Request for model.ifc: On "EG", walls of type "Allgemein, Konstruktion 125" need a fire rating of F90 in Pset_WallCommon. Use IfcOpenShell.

First a look at what the model holds.

```python
import ifcopenshell
import ifcopenshell.util.element

model = ifcopenshell.open("model.ifc")
print(model.schema)
storey = next(s for s in model.by_type("IfcBuildingStorey") if s.Name == "EG")
walls = [e for e in ifcopenshell.util.element.get_decomposition(storey) if e.is_a("IfcWall")]
seen = {}
for e in walls:
    element_type = ifcopenshell.util.element.get_type(e)
    key = (element_type.Name if element_type != e and element_type else None, ifcopenshell.util.element.get_pset(e, "Pset_WallCommon", "FireRating"))
    seen[key] = seen.get(key, 0) + 1
for (name, value), count in sorted(seen.items(), key=str):
    print(count, "x", name, "|", value)
```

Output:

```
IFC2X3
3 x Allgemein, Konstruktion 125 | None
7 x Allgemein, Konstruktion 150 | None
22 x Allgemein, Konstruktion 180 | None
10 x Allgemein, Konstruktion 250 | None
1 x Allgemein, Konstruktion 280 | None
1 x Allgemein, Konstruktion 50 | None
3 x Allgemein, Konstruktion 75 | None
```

```python
import ifcopenshell
import ifcopenshell.api.pset
import ifcopenshell.util.element

model = ifcopenshell.open("model.ifc")

storey = next(s for s in model.by_type("IfcBuildingStorey") if s.Name == "EG")
walls = [e for e in ifcopenshell.util.element.get_decomposition(storey) if e.is_a("IfcWall")]

count = 0
for e in walls:
    element_type = ifcopenshell.util.element.get_type(e)
    if element_type in (None, e) or element_type.Name != "Allgemein, Konstruktion 125":
        continue
    # add_pset returns the element's existing set when there is one.
    pset = ifcopenshell.api.pset.add_pset(model, product=e, name="Pset_WallCommon")
    ifcopenshell.api.pset.edit_pset(model, pset=pset, properties={"FireRating": "F90"})
    count += 1

print(count, "walls updated")

model.write("model_updated.ifc")
```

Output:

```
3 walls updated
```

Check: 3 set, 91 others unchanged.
